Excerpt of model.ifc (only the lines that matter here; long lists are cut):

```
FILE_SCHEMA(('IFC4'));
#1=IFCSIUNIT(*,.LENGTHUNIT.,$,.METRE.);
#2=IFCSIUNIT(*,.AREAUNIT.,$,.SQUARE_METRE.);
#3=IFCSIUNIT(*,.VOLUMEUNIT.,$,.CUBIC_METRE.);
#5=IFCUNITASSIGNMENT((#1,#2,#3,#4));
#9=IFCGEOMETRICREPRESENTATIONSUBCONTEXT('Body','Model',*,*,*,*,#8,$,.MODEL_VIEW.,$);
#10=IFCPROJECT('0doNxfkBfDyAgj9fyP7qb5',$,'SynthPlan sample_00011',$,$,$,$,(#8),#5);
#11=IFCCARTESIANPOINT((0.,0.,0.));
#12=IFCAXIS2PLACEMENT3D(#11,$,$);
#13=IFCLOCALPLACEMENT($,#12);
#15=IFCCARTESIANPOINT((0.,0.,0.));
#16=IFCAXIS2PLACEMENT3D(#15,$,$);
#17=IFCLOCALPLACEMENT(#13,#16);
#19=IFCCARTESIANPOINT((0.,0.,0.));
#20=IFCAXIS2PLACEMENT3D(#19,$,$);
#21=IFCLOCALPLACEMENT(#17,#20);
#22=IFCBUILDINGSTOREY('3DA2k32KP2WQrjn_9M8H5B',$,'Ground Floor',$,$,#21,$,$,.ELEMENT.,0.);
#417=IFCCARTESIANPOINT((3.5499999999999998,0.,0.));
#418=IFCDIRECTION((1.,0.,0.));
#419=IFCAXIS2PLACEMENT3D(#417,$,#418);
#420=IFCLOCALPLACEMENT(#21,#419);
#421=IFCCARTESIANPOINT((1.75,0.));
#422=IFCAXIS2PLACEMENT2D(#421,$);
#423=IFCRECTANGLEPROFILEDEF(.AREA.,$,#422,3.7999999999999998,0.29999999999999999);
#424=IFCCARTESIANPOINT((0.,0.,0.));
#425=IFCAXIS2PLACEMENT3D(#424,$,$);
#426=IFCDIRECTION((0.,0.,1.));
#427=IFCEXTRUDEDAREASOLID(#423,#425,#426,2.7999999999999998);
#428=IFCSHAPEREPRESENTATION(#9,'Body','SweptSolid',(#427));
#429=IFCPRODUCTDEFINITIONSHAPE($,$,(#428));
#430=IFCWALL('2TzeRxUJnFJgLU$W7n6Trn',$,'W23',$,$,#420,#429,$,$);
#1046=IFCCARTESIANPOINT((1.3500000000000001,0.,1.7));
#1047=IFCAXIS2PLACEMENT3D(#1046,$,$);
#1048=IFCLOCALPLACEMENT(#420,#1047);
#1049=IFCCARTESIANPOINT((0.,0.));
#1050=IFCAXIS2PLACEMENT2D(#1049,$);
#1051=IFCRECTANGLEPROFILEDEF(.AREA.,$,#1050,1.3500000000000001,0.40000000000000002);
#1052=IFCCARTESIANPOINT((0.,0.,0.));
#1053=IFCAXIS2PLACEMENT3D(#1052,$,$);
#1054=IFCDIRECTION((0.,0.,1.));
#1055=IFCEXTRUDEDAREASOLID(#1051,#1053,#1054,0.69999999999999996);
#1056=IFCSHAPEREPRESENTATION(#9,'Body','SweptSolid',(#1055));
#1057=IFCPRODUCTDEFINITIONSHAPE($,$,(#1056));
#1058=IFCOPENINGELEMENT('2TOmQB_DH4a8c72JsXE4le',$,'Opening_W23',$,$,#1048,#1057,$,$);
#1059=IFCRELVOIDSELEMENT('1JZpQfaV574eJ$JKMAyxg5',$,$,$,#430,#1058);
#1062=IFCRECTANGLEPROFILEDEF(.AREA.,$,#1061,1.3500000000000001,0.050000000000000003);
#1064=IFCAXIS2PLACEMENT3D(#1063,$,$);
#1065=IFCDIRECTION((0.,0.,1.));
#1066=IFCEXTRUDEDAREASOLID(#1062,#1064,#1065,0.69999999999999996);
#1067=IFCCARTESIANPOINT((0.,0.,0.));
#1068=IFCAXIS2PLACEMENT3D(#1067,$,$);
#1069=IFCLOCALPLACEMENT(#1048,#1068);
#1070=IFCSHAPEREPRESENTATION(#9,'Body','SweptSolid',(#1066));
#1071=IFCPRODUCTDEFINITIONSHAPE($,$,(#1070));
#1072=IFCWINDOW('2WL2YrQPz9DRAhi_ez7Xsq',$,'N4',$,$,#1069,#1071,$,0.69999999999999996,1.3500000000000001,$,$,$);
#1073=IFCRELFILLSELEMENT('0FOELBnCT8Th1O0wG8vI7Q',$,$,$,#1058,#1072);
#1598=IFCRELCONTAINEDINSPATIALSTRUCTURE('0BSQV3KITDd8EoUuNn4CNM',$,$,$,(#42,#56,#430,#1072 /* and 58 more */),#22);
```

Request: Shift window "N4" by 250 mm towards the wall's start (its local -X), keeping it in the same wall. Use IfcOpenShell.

```python
import ifcopenshell
import ifcopenshell.api.geometry
import ifcopenshell.util.placement
import ifcopenshell.util.unit

model = ifcopenshell.open("model.ifc")
unit_scale = ifcopenshell.util.unit.calculate_unit_scale(model)

window = model.by_guid("2WL2YrQPz9DRAhi_ez7Xsq")
opening = window.FillsVoids[0].RelatingOpeningElement
wall = opening.VoidsElements[0].RelatingBuildingElement

wall_matrix = ifcopenshell.util.placement.get_local_placement(wall.ObjectPlacement)
shift = wall_matrix[:3, 0] * -0.25 / unit_scale
before = ifcopenshell.util.placement.get_local_placement(window.ObjectPlacement)[:3, 3].copy()

# The window is placed relative to its opening, so it follows when the opening moves.
matrix = ifcopenshell.util.placement.get_local_placement(opening.ObjectPlacement)
matrix[:3, 3] += shift
ifcopenshell.api.geometry.edit_object_placement(
    model, product=opening, matrix=matrix, is_si=False, should_transform_children=True
)

after = ifcopenshell.util.placement.get_local_placement(window.ObjectPlacement)[:3, 3]
print("window moved by", (after - before).round(3) + 0.0)

model.write("model_updated.ifc")
```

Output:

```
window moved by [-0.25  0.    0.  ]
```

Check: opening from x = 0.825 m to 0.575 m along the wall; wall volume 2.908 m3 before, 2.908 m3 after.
